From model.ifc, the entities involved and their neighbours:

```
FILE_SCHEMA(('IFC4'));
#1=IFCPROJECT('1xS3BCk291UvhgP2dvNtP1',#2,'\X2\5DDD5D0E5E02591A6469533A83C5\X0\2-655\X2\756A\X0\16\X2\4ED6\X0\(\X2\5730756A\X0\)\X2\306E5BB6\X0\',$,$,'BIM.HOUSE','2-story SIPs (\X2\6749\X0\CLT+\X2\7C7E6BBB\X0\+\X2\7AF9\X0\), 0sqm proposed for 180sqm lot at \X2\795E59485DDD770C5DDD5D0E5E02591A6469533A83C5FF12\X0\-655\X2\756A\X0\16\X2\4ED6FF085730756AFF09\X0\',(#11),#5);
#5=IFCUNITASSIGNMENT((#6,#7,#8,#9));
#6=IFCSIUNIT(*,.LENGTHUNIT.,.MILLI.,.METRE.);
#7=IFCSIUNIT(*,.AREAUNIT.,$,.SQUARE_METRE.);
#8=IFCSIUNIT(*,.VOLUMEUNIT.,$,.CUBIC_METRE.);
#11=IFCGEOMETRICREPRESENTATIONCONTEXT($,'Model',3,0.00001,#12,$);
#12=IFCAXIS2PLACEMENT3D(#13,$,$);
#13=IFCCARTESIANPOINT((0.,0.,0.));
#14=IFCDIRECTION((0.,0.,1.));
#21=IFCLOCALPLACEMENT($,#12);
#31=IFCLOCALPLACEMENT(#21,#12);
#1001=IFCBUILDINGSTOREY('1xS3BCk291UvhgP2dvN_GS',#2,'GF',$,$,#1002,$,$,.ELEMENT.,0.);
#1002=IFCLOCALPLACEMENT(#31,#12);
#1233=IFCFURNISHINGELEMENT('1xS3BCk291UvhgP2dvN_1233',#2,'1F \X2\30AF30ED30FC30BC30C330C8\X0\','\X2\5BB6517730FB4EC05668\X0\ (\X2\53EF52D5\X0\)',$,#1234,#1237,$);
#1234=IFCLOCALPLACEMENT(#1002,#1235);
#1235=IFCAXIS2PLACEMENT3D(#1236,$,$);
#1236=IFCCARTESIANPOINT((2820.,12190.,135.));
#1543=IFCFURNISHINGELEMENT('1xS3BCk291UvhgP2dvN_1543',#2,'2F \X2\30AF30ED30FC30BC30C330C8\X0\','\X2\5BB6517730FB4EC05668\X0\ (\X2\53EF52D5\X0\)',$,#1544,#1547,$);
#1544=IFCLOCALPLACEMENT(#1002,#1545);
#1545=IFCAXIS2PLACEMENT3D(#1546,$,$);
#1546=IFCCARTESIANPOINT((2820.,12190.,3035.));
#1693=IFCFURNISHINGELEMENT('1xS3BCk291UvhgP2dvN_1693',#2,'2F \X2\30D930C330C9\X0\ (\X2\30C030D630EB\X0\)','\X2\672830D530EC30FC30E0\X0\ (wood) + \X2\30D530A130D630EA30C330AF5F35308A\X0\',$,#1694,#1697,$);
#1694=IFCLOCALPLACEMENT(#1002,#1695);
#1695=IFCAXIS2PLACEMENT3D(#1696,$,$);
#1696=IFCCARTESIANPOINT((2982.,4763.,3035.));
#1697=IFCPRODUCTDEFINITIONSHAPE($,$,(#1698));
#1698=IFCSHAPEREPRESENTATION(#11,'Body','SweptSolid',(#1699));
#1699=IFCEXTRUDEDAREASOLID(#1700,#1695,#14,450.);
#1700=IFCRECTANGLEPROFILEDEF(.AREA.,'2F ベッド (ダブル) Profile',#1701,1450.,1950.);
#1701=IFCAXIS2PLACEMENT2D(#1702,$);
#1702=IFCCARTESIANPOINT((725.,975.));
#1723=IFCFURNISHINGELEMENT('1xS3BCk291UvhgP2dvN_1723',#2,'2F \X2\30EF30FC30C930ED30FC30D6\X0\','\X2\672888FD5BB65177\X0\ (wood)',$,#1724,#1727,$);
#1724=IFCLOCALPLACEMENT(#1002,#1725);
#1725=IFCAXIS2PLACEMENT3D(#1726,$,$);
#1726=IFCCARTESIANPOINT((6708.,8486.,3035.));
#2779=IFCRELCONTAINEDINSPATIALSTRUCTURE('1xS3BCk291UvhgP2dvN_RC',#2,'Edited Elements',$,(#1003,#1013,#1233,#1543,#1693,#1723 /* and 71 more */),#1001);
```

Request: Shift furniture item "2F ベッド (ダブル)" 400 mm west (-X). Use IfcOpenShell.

```python
import ifcopenshell
import ifcopenshell.api.geometry
import ifcopenshell.util.placement

model = ifcopenshell.open("model.ifc")

item = model.by_guid("1xS3BCk291UvhgP2dvN_1693")
matrix = ifcopenshell.util.placement.get_local_placement(item.ObjectPlacement)
matrix[0, 3] -= 400.0
ifcopenshell.api.geometry.edit_object_placement(model, product=item, matrix=matrix, is_si=False)

print(ifcopenshell.util.placement.get_local_placement(item.ObjectPlacement).round(3) + 0.0)

model.write("model_edited.ifc")
```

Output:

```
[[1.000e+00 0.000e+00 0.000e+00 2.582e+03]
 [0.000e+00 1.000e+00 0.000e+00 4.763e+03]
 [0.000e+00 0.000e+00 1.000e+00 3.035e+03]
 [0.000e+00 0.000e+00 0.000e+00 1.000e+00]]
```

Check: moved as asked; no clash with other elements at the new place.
